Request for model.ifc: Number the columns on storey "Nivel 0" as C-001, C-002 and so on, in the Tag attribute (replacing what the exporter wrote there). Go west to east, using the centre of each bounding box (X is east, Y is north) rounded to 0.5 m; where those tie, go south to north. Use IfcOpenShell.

First a look at what the model holds.

```python
import ifcopenshell
import ifcopenshell.util.element
import ifcopenshell.util.placement

model = ifcopenshell.open("model.ifc")
print(model.schema)
storey = next(s for s in model.by_type("IfcBuildingStorey") if s.Name == "Nivel 0")
columns = [e for e in ifcopenshell.util.element.get_decomposition(storey) if e.is_a("IfcColumn")]
for e in sorted(columns, key=lambda e: e.id()):
    origin = ifcopenshell.util.placement.get_local_placement(e.ObjectPlacement)[:3, 3]
    print(e.id(), e.Tag, e.Name, origin.round(2) + 0.0, sep=" | ")
```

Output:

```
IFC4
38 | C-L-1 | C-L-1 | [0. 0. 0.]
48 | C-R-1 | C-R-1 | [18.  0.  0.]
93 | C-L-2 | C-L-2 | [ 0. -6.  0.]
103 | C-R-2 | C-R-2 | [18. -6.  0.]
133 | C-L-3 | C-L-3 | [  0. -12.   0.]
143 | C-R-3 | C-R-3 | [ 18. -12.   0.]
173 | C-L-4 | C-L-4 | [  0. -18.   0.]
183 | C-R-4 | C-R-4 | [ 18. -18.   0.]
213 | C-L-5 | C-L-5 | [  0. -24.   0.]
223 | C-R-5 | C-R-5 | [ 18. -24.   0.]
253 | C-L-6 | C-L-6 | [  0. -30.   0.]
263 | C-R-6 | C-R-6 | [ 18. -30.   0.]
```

```python
import ifcopenshell
import ifcopenshell.geom
import ifcopenshell.util.element
import ifcopenshell.util.shape

model = ifcopenshell.open("model.ifc")
settings = ifcopenshell.geom.settings()
settings.set("use-world-coords", True)


def centre(element):
    shape = ifcopenshell.geom.create_shape(settings, element)
    return ifcopenshell.util.shape.get_bbox_centroid(shape.geometry)


storey = next(s for s in model.by_type("IfcBuildingStorey") if s.Name == "Nivel 0")
columns = [e for e in ifcopenshell.util.element.get_decomposition(storey) if e.is_a("IfcColumn")]

# Insertion points can sit at a corner or the storey origin, so sort by the geometry (in metres).
centres = {e: centre(e) for e in columns}
columns.sort(key=lambda e: (round(centres[e][0] / 0.5), centres[e][1]))

for i, e in enumerate(columns, start=1):
    number = f"C-0{i:02d}"
    e.Tag = number
    print(e.id(), number)

model.write("model_v2.ifc")
```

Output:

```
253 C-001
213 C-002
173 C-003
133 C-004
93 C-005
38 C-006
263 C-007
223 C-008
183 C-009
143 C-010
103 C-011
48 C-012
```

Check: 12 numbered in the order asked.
